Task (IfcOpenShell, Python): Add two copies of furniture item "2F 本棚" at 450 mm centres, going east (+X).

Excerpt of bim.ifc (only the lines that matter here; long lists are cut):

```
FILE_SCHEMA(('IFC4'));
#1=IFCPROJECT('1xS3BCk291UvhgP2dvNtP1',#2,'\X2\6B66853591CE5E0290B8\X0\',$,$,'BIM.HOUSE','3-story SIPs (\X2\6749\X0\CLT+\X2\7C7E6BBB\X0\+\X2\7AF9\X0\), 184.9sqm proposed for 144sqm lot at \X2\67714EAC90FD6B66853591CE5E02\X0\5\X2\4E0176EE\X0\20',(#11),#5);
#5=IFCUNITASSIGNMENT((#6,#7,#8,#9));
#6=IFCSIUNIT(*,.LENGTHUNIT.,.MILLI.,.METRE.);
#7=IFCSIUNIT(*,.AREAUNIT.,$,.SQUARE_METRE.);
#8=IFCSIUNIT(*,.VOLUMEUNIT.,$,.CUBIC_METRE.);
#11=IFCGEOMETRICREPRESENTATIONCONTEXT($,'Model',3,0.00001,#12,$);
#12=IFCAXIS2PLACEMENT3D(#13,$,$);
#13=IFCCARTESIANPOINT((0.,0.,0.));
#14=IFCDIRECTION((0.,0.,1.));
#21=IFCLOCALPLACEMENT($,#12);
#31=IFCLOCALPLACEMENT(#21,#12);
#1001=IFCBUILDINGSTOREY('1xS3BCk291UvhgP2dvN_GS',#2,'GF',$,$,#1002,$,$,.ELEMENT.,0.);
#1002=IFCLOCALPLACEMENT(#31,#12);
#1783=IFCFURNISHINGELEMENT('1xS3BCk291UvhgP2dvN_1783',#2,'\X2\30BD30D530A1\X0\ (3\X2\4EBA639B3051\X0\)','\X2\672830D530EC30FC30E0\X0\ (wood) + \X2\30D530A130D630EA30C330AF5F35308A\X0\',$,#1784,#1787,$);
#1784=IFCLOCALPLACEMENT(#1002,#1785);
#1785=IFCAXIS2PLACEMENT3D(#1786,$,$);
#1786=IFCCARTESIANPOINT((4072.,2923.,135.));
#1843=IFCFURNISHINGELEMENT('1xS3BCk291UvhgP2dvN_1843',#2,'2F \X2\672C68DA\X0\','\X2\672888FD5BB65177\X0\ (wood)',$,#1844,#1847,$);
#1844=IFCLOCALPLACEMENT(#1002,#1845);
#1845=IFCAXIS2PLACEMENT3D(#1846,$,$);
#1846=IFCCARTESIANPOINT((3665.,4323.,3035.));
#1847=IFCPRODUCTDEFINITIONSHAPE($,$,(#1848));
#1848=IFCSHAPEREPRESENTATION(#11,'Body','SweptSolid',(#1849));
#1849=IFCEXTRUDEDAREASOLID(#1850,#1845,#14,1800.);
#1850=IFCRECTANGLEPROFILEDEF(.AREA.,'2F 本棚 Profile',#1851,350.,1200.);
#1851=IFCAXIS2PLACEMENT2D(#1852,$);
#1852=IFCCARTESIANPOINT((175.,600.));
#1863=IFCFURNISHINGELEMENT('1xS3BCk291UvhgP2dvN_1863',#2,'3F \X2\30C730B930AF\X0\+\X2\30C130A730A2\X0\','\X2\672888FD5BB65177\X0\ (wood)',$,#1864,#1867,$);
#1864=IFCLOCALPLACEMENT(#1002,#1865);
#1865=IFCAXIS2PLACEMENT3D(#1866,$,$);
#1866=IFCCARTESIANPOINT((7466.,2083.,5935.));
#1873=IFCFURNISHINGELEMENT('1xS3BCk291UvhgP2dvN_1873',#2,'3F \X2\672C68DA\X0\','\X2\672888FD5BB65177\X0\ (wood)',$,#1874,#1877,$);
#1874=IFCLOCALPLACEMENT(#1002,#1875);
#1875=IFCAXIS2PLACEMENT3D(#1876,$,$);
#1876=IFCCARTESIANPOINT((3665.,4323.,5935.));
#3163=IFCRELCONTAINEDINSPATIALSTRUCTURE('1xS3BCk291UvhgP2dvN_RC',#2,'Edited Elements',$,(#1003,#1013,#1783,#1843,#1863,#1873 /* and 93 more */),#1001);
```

```python
import numpy as np
import ifcopenshell
import ifcopenshell.api.geometry
import ifcopenshell.api.root
import ifcopenshell.util.element
import ifcopenshell.util.placement

model = ifcopenshell.open("bim.ifc")


def reuse_history(source, copy):
    """copy_class also copies each property set's owner history, people and application; keep the originals."""
    for rel in copy.IsDefinedBy:
        if rel.is_a("IfcRelDefinesByProperties") and (history := rel.RelatingPropertyDefinition.OwnerHistory):
            rel.RelatingPropertyDefinition.OwnerHistory = source.OwnerHistory
            ifcopenshell.util.element.remove_deep2(model, history)


source = model.by_guid("1xS3BCk291UvhgP2dvN_1843")
base = ifcopenshell.util.placement.get_local_placement(source.ObjectPlacement)
step = np.array([1.0, 0.0, 0.0]) * 450.0

for i in range(1, 3):
    copy = ifcopenshell.api.root.copy_class(model, product=source)
    copy.Representation = ifcopenshell.util.element.copy_deep(
        model, source.Representation, exclude=["IfcGeometricRepresentationContext", "IfcRepresentationMap"]
    )
    reuse_history(source, copy)
    matrix = base.copy()
    matrix[:3, 3] += i * step
    print("added at", matrix[:3, 3].round(3) + 0.0)
    ifcopenshell.api.geometry.edit_object_placement(model, product=copy, matrix=matrix, is_si=False)

model.write("bim_v2.ifc")
```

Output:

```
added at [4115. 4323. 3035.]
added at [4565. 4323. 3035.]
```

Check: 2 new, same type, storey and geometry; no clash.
